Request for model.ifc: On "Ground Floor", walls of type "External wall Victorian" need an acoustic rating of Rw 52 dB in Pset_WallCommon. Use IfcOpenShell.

First a look at what the model holds.

```python
import ifcopenshell
import ifcopenshell.util.element

model = ifcopenshell.open("model.ifc")
print(model.schema)
storey = next(s for s in model.by_type("IfcBuildingStorey") if s.Name == "Ground Floor")
walls = [e for e in ifcopenshell.util.element.get_decomposition(storey) if e.is_a("IfcWall")]
seen = {}
for e in walls:
    element_type = ifcopenshell.util.element.get_type(e)
    key = (element_type.Name if element_type != e and element_type else None, ifcopenshell.util.element.get_pset(e, "Pset_WallCommon", "AcousticRating"))
    seen[key] = seen.get(key, 0) + 1
for (name, value), count in sorted(seen.items(), key=str):
    print(count, "x", name, "|", value)
```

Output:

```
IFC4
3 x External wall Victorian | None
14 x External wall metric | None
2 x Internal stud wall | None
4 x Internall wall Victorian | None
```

```python
import ifcopenshell
import ifcopenshell.api.pset
import ifcopenshell.util.element

model = ifcopenshell.open("model.ifc")

storey = next(s for s in model.by_type("IfcBuildingStorey") if s.Name == "Ground Floor")
walls = [e for e in ifcopenshell.util.element.get_decomposition(storey) if e.is_a("IfcWall")]

count = 0
for e in walls:
    element_type = ifcopenshell.util.element.get_type(e)
    if element_type in (None, e) or element_type.Name != "External wall Victorian":
        continue
    # add_pset returns the element's existing set when there is one.
    pset = ifcopenshell.api.pset.add_pset(model, product=e, name="Pset_WallCommon")
    ifcopenshell.api.pset.edit_pset(model, pset=pset, properties={"AcousticRating": "Rw 52 dB"})
    count += 1

print(count, "walls updated")

model.write("model_edited.ifc")
```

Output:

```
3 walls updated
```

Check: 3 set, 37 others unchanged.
